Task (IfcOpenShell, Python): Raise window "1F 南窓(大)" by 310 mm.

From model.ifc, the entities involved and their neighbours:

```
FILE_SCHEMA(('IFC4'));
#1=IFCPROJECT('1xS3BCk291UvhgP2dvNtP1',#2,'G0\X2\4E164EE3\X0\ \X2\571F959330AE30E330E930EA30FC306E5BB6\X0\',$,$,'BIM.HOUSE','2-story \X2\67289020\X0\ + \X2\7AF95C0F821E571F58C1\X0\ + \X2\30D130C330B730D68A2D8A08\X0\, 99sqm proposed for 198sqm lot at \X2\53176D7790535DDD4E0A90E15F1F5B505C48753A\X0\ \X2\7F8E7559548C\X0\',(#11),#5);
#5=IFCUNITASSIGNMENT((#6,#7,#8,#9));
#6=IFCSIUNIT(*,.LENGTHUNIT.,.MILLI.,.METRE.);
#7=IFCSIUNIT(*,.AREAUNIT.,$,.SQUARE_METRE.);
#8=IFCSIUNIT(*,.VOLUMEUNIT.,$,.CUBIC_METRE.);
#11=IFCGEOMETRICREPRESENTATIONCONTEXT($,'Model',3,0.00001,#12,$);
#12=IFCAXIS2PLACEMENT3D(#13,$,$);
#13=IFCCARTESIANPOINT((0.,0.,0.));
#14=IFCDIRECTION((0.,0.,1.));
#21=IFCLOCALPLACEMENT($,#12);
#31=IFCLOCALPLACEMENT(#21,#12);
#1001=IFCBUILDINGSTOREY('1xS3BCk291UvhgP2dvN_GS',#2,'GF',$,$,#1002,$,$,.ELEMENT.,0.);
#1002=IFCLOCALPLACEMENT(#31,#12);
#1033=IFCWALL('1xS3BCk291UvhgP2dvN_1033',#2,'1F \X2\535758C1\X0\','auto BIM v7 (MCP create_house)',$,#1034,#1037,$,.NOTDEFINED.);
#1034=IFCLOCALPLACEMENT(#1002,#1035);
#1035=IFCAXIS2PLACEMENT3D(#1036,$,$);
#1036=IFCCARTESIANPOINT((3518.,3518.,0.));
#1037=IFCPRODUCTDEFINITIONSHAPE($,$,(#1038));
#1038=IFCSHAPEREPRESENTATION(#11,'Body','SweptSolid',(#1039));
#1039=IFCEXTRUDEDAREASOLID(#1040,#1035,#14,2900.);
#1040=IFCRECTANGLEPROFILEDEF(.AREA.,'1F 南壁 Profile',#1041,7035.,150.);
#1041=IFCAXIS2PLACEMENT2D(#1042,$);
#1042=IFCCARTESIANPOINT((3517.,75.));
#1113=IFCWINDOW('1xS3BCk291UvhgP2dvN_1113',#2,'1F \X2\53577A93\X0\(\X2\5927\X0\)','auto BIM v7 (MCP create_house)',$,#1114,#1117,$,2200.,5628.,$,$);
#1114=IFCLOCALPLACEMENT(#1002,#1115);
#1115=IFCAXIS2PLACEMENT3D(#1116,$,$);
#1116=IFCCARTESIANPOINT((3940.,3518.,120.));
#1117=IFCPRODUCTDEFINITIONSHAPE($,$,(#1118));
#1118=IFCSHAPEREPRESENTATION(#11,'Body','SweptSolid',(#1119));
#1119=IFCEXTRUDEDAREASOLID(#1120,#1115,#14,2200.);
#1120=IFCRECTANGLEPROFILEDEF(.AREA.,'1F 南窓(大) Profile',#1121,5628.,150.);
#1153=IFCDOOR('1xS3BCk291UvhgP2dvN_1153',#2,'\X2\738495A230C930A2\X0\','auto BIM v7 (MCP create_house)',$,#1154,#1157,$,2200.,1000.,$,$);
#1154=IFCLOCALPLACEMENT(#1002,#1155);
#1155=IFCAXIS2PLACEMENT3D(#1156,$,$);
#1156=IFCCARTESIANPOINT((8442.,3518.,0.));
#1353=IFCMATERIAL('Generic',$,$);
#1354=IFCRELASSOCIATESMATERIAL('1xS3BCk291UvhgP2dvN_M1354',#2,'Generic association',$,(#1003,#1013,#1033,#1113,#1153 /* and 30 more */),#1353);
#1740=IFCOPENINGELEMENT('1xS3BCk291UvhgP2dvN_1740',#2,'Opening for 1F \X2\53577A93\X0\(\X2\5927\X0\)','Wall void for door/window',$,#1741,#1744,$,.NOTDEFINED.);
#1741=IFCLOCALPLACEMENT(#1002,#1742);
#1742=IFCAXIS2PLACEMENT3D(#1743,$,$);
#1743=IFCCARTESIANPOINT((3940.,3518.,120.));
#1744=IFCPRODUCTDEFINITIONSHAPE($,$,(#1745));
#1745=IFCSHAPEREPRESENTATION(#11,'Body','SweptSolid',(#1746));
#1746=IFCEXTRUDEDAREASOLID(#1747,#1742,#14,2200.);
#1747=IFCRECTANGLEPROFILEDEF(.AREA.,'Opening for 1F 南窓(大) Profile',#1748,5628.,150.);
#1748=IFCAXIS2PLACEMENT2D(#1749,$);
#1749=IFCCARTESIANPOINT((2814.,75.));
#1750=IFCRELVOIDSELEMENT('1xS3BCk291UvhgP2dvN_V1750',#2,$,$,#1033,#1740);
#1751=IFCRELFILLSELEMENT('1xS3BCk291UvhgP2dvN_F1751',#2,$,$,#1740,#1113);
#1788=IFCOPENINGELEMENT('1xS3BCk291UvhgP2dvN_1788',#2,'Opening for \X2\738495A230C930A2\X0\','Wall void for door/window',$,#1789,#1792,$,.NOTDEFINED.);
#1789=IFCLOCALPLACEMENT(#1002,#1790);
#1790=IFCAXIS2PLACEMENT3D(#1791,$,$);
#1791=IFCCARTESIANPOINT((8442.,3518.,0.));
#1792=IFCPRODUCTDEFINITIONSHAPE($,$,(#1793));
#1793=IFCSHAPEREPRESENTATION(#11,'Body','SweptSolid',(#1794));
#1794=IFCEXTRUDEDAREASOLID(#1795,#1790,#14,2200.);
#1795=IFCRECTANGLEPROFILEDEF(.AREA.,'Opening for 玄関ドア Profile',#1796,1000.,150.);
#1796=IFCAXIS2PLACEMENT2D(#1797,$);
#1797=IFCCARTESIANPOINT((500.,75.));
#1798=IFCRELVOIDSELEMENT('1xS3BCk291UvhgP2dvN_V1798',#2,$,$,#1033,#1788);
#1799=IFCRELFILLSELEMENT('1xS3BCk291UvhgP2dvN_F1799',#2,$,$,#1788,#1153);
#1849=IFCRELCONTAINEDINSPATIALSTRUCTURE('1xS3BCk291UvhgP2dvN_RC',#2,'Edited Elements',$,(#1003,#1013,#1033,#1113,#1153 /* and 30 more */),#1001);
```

```python
import numpy as np
import ifcopenshell
import ifcopenshell.api.geometry
import ifcopenshell.util.placement
import ifcopenshell.util.unit

model = ifcopenshell.open("model.ifc")
unit_scale = ifcopenshell.util.unit.calculate_unit_scale(model)

window = model.by_id(1113)
opening = window.FillsVoids[0].RelatingOpeningElement
dz = 0.31 / unit_scale

shift = np.array([0.0, 0.0, dz])
# The window is not placed relative to its opening, so move both.
for product in (opening, window):
    matrix = ifcopenshell.util.placement.get_local_placement(product.ObjectPlacement)
    matrix[:3, 3] += shift
    ifcopenshell.api.geometry.edit_object_placement(model, product=product, matrix=matrix, is_si=False)

print(f"moved by {dz * unit_scale:+.3f} m")

model.write("model_edited.ifc")
```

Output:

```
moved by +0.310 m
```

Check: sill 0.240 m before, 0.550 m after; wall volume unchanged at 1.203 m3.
